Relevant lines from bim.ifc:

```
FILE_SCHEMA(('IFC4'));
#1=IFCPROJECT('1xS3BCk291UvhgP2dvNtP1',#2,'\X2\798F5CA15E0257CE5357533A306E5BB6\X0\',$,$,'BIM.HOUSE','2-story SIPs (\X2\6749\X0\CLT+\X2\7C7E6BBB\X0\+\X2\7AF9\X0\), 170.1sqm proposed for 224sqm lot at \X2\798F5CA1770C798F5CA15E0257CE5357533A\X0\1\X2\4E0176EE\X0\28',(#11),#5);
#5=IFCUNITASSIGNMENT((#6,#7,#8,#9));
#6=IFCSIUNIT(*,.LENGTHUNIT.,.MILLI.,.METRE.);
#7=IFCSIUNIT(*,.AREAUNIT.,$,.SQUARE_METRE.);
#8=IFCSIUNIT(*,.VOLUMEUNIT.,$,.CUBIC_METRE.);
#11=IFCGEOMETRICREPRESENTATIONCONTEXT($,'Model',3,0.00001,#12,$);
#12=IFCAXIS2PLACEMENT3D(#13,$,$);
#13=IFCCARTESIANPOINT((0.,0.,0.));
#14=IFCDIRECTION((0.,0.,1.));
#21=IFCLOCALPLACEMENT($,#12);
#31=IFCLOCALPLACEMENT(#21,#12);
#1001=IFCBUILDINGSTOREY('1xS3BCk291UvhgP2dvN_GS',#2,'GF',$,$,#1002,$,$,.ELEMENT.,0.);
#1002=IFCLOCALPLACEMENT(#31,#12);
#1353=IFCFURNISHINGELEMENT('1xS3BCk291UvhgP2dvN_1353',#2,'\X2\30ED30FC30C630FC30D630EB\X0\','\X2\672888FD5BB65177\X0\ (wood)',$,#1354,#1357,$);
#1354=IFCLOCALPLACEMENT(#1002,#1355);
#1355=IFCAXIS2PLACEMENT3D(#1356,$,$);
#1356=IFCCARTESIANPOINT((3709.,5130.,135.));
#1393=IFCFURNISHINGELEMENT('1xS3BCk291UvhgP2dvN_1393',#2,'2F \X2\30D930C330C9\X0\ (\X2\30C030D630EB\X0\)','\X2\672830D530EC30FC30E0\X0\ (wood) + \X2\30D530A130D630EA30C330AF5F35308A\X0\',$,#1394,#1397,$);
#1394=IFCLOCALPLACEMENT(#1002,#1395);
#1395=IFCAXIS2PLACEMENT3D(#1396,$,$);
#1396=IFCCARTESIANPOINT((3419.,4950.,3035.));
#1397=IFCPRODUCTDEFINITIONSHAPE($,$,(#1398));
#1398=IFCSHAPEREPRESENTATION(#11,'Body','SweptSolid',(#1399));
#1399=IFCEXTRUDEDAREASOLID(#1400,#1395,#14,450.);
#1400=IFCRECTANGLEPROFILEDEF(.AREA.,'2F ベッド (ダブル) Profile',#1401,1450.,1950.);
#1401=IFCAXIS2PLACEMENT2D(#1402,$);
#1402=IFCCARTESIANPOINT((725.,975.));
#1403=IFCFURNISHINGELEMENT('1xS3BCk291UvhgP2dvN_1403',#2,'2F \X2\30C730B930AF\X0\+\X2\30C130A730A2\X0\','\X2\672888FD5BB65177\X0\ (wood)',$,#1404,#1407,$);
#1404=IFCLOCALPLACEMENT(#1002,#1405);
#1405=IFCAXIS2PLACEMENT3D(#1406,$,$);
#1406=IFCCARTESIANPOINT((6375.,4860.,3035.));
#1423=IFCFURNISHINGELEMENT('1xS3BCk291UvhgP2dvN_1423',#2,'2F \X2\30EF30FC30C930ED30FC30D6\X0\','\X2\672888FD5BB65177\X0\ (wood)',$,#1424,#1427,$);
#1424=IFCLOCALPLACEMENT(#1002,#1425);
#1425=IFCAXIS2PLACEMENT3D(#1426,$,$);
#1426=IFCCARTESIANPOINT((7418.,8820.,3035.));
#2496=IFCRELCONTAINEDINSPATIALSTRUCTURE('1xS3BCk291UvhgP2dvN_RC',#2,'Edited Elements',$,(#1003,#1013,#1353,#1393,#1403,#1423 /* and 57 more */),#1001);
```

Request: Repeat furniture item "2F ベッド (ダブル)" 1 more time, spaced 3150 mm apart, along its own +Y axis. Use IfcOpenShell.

```python
import ifcopenshell
import ifcopenshell.api.geometry
import ifcopenshell.api.root
import ifcopenshell.util.element
import ifcopenshell.util.placement

model = ifcopenshell.open("bim.ifc")


def reuse_history(source, copy):
    """copy_class also copies each property set's owner history, people and application; keep the originals."""
    for rel in copy.IsDefinedBy:
        if rel.is_a("IfcRelDefinesByProperties") and (history := rel.RelatingPropertyDefinition.OwnerHistory):
            rel.RelatingPropertyDefinition.OwnerHistory = source.OwnerHistory
            ifcopenshell.util.element.remove_deep2(model, history)


source = model.by_guid("1xS3BCk291UvhgP2dvN_1393")
base = ifcopenshell.util.placement.get_local_placement(source.ObjectPlacement)
step = base[:3, 1] * 3150.0

for i in range(1, 2):
    copy = ifcopenshell.api.root.copy_class(model, product=source)
    copy.Representation = ifcopenshell.util.element.copy_deep(
        model, source.Representation, exclude=["IfcGeometricRepresentationContext", "IfcRepresentationMap"]
    )
    reuse_history(source, copy)
    matrix = base.copy()
    matrix[:3, 3] += i * step
    print("added at", matrix[:3, 3].round(3) + 0.0)
    ifcopenshell.api.geometry.edit_object_placement(model, product=copy, matrix=matrix, is_si=False)

model.write("bim-out.ifc")
```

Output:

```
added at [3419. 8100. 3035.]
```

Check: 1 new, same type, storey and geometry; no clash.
